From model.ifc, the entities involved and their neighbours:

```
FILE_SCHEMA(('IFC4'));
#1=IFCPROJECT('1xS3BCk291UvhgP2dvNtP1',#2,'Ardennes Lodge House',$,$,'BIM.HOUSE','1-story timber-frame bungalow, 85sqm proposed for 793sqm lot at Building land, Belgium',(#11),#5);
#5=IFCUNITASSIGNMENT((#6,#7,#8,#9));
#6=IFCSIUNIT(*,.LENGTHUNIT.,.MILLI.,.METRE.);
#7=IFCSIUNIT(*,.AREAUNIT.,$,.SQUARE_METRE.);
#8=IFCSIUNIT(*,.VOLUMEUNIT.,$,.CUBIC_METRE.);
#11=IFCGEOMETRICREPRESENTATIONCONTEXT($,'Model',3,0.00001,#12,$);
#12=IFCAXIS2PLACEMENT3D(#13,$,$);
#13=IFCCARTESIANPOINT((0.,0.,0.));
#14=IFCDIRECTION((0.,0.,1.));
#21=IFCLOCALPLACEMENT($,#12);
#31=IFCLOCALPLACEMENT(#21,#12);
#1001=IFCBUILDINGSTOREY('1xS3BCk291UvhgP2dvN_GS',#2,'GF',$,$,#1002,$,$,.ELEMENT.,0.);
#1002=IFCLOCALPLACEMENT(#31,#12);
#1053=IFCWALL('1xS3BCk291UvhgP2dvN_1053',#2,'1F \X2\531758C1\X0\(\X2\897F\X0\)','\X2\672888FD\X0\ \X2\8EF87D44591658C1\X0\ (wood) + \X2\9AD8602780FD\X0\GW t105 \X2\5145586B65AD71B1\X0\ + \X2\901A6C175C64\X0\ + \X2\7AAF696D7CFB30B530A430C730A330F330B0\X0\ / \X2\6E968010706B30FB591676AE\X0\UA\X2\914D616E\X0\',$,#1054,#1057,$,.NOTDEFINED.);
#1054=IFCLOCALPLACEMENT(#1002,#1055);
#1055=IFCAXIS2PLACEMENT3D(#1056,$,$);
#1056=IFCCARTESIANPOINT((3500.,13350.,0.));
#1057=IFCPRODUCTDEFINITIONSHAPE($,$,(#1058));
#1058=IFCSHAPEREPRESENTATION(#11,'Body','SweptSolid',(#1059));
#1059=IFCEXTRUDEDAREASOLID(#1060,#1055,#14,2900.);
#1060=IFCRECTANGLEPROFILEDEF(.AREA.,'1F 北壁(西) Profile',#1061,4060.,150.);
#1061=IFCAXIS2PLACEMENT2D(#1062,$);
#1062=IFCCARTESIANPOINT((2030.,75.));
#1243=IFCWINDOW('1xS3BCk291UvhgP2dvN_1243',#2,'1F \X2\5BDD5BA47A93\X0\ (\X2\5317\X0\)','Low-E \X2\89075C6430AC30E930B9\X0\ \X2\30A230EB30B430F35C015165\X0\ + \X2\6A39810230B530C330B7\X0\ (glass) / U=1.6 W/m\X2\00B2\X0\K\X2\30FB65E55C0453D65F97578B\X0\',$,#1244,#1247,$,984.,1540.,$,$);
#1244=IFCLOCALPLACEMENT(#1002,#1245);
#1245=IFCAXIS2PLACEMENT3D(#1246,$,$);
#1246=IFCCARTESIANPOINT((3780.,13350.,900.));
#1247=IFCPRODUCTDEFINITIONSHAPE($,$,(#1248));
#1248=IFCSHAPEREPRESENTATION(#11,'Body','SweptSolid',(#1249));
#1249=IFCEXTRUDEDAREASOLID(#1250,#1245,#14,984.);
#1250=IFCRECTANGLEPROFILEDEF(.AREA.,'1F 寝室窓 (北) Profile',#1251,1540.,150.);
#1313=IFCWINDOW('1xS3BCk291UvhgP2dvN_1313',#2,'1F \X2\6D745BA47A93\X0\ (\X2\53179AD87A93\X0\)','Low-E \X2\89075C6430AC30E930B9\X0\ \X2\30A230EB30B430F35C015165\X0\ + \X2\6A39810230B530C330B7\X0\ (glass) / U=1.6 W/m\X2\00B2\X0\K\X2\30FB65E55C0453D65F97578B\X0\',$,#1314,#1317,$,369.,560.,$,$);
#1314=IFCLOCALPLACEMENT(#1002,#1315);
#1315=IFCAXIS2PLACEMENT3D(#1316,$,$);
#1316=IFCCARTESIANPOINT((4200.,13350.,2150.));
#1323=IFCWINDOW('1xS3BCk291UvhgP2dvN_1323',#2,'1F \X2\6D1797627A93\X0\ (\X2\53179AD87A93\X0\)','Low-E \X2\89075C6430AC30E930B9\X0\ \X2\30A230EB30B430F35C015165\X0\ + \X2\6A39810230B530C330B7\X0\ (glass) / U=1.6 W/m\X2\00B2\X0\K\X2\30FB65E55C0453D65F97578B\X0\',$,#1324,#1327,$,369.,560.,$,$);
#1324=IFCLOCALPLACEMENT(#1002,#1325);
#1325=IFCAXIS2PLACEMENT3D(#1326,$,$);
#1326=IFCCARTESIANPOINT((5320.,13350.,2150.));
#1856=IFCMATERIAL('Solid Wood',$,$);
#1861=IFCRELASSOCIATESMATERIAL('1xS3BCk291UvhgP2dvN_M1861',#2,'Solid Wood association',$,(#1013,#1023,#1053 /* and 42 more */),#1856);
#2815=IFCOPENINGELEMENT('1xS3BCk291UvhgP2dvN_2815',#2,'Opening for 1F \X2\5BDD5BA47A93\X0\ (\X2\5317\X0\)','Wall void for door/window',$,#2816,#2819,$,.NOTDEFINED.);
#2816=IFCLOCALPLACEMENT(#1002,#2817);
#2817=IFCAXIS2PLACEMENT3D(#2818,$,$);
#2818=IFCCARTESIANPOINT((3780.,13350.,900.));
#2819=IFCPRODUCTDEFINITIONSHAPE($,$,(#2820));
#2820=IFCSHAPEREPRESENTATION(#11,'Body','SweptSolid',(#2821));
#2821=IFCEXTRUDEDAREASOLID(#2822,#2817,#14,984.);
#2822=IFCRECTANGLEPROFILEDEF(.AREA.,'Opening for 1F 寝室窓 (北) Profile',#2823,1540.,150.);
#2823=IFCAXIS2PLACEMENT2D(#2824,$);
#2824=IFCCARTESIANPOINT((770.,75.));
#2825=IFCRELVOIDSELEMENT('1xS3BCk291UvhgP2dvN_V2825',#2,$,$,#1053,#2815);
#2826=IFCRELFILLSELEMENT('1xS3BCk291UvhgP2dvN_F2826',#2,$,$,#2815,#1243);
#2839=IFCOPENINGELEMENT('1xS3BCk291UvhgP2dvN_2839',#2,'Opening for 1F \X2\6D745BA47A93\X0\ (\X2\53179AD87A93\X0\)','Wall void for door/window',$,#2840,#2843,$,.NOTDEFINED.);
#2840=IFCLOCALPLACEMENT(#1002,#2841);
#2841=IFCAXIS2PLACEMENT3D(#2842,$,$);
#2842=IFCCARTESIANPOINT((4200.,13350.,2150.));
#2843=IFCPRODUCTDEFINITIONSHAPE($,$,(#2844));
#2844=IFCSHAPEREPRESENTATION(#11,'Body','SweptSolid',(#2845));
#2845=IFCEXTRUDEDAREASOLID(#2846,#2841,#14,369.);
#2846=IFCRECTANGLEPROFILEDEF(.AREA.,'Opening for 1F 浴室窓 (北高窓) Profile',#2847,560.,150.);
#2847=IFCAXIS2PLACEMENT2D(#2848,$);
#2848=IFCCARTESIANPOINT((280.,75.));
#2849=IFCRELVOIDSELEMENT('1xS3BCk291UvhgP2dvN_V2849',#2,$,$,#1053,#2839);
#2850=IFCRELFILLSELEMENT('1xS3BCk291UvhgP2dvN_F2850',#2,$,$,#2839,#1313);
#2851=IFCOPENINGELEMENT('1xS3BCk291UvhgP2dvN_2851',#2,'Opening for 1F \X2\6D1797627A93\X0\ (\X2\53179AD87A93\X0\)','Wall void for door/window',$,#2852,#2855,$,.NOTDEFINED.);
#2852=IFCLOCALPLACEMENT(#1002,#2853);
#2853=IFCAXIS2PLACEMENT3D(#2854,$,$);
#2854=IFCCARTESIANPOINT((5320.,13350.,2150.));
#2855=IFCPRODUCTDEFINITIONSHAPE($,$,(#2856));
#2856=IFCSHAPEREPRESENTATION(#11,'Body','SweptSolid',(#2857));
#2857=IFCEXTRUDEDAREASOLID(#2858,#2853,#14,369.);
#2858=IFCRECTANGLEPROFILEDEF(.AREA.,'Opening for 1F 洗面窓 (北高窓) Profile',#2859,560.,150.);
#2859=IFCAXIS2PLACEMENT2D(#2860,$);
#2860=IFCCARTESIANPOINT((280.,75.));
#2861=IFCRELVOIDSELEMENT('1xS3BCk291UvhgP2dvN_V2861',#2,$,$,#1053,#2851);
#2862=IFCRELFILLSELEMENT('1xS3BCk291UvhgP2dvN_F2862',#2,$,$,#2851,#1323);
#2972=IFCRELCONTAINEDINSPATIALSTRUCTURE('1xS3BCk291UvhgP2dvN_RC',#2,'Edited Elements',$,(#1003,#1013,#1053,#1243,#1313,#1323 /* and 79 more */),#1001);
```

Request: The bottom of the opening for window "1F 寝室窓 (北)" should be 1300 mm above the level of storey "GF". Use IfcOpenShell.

```python
import numpy as np
import ifcopenshell
import ifcopenshell.api.geometry
import ifcopenshell.geom
import ifcopenshell.util.element
import ifcopenshell.util.placement
import ifcopenshell.util.shape
import ifcopenshell.util.unit

model = ifcopenshell.open("model.ifc")
unit_scale = ifcopenshell.util.unit.calculate_unit_scale(model)

window = model.by_guid("1xS3BCk291UvhgP2dvN_1243")
opening = window.FillsVoids[0].RelatingOpeningElement
storey = ifcopenshell.util.element.get_container(window, ifc_class="IfcBuildingStorey")
level = ifcopenshell.util.placement.get_local_placement(storey.ObjectPlacement)[2, 3]

# The opening's origin need not be at the sill, so measure its lowest point.
shape = ifcopenshell.geom.create_shape(ifcopenshell.geom.settings(), opening)
bottom = ifcopenshell.util.shape.get_shape_bottom_elevation(shape, shape.geometry) / unit_scale
dz = level + 1.3 / unit_scale - bottom

shift = np.array([0.0, 0.0, dz])
# The window is not placed relative to its opening, so move both.
for product in (opening, window):
    matrix = ifcopenshell.util.placement.get_local_placement(product.ObjectPlacement)
    matrix[:3, 3] += shift
    ifcopenshell.api.geometry.edit_object_placement(model, product=product, matrix=matrix, is_si=False)

print(f"moved by {dz * unit_scale:+.3f} m")

model.write("model_v2.ifc")
```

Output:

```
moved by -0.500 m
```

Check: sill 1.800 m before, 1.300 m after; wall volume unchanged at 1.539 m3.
